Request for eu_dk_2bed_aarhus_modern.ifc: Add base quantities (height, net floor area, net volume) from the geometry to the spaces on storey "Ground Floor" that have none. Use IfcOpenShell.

First a look at what the model holds.

```python
import ifcopenshell
import ifcopenshell.util.element
import ifcopenshell.util.unit

model = ifcopenshell.open("eu_dk_2bed_aarhus_modern.ifc")
print(model.schema)
for unit_type in ("LENGTHUNIT", "AREAUNIT", "VOLUMEUNIT"):
    print(unit_type, ifcopenshell.util.unit.calculate_unit_scale(model, unit_type))
storey = next(s for s in model.by_type("IfcBuildingStorey") if s.Name == "Ground Floor")
spaces = [e for e in ifcopenshell.util.element.get_decomposition(storey) if e.is_a("IfcSpace")]
for e in sorted(spaces, key=lambda e: e.id()):
    print(e.id(), e.is_a(), e.Name, list(ifcopenshell.util.element.get_psets(e, qtos_only=True)), sep=" | ")
```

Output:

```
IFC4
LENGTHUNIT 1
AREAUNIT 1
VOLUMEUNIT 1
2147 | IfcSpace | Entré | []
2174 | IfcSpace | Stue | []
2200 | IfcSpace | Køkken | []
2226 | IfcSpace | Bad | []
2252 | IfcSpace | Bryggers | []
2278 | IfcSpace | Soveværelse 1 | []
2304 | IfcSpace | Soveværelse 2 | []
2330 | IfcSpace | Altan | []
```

```python
import ifcopenshell
import ifcopenshell.api.pset
import ifcopenshell.geom
import ifcopenshell.util.element
import ifcopenshell.util.shape
import ifcopenshell.util.unit

model = ifcopenshell.open("eu_dk_2bed_aarhus_modern.ifc")
unit_scale = ifcopenshell.util.unit.calculate_unit_scale(model)
area_scale = ifcopenshell.util.unit.calculate_unit_scale(model, "AREAUNIT")
volume_scale = ifcopenshell.util.unit.calculate_unit_scale(model, "VOLUMEUNIT")
settings = ifcopenshell.geom.settings()

storey = next(s for s in model.by_type("IfcBuildingStorey") if s.Name == "Ground Floor")
spaces = [e for e in ifcopenshell.util.element.get_decomposition(storey) if e.is_a("IfcSpace")]

for e in sorted(spaces, key=lambda e: e.id()):
    if ifcopenshell.util.element.get_psets(e, qtos_only=True, should_inherit=False):
        continue
    # Geometry comes back in metres, in the element's own axes.
    shape = ifcopenshell.geom.create_shape(settings, e)
    values = {
        "Height": ifcopenshell.util.shape.get_z(shape.geometry) / unit_scale,
        "NetFloorArea": ifcopenshell.util.shape.get_footprint_area(shape.geometry) / area_scale,
        "NetVolume": ifcopenshell.util.shape.get_volume(shape.geometry) / volume_scale,
    }
    qto = ifcopenshell.api.pset.add_qto(model, product=e, name="Qto_SpaceBaseQuantities")
    ifcopenshell.api.pset.edit_qto(model, qto=qto, properties=values)
    print(e.id(), {k: round(v, 3) for k, v in values.items()})

model.write("eu_dk_2bed_aarhus_modern_edited.ifc")
```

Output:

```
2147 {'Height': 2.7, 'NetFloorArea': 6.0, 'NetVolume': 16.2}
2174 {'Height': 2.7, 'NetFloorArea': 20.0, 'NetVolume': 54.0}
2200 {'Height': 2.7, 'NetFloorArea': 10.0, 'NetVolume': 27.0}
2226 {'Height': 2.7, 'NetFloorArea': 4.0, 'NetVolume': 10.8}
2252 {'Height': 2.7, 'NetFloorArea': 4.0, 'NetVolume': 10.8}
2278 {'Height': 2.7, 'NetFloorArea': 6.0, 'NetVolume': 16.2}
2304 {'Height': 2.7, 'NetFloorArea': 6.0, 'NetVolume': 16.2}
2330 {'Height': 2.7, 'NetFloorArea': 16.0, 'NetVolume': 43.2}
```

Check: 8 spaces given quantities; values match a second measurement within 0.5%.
